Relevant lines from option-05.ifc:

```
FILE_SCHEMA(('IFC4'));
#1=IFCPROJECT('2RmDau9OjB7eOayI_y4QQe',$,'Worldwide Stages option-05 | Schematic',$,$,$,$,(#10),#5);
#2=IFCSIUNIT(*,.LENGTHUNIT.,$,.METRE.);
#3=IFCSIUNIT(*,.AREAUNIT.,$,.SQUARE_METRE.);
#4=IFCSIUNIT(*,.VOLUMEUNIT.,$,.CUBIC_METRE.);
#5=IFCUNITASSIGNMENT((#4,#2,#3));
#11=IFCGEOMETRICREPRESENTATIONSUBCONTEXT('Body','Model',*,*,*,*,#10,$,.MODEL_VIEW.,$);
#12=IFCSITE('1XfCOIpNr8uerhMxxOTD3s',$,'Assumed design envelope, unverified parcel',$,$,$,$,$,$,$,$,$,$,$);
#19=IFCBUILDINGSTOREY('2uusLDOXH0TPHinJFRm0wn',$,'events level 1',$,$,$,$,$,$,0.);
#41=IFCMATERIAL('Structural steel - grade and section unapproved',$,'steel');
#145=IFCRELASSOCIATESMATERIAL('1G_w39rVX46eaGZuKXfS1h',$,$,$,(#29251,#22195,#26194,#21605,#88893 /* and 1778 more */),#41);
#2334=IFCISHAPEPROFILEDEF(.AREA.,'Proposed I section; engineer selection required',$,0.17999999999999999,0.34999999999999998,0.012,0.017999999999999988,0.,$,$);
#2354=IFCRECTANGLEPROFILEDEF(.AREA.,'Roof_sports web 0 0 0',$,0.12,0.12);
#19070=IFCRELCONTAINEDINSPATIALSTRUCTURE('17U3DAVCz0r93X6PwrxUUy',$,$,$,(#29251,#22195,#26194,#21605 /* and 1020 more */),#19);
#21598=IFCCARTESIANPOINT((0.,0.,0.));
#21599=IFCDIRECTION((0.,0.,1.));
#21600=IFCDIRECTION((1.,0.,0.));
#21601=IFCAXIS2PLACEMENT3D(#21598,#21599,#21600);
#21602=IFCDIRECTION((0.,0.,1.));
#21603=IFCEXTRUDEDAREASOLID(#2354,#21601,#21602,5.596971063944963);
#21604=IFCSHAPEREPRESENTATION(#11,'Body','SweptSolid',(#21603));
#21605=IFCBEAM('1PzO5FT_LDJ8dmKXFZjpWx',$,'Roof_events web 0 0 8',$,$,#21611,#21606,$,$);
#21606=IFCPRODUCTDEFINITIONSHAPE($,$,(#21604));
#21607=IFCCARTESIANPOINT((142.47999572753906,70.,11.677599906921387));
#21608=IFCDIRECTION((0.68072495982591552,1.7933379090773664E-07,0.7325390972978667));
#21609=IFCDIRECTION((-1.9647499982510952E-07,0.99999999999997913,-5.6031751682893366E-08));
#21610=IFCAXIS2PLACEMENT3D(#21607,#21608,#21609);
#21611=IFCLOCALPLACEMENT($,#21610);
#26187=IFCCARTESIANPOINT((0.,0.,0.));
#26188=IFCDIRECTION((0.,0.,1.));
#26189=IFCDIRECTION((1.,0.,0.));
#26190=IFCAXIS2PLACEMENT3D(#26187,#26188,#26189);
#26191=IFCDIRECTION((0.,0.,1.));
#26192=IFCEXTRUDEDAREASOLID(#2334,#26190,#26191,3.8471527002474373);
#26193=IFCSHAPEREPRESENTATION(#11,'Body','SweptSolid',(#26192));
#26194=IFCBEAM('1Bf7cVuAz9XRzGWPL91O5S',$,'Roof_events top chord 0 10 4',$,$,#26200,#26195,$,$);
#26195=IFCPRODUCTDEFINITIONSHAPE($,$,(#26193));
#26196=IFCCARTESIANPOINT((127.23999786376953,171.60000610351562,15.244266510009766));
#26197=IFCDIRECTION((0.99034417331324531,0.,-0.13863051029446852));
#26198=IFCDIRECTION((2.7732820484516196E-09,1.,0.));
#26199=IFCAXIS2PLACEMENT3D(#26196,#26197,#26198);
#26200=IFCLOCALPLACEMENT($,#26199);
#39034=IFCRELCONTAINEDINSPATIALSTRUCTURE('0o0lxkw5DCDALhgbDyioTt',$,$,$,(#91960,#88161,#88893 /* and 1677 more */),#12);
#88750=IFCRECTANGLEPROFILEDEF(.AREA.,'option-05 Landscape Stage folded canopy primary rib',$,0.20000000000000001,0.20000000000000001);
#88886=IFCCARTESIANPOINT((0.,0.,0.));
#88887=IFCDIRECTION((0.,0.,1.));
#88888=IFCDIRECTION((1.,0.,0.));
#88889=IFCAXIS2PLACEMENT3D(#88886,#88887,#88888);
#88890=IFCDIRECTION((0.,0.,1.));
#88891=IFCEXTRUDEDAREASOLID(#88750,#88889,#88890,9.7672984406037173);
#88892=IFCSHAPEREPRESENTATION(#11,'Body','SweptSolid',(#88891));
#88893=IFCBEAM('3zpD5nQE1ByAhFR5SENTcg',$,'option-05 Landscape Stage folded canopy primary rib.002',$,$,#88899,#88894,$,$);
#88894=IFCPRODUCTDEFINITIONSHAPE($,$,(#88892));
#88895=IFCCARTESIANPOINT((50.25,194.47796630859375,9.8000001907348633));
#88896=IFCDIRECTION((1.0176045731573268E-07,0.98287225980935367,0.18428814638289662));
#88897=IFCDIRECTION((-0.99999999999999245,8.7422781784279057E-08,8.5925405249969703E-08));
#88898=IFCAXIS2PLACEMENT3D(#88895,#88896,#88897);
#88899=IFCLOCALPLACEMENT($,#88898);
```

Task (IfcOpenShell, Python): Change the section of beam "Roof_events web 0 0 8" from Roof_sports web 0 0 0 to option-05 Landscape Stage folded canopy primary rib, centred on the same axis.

```python
import ifcopenshell
import ifcopenshell.util.element
import ifcopenshell.util.representation

model = ifcopenshell.open("option-05.ifc")

member = model.by_guid("1PzO5FT_LDJ8dmKXFZjpWx")
source = next(p for p in model.by_type("IfcRectangleProfileDef") if p.ProfileName == "option-05 Landscape Stage folded canopy primary rib")

body = ifcopenshell.util.representation.get_representation(member, "Model", "Body")
solid = body.Items[0]
old_profile = solid.SweptArea

# Copy the section's sizes but keep this member's own profile position.
profile = ifcopenshell.util.element.copy(model, source)
profile.Position = old_profile.Position
solid.SweptArea = profile
if not model.get_total_inverses(old_profile):
    ifcopenshell.util.element.remove_deep2(model, old_profile)

print(solid.SweptArea)

model.write("option-05_edited.ifc")
```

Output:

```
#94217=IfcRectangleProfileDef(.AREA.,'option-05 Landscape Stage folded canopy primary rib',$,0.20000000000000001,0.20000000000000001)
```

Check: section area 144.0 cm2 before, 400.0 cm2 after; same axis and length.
